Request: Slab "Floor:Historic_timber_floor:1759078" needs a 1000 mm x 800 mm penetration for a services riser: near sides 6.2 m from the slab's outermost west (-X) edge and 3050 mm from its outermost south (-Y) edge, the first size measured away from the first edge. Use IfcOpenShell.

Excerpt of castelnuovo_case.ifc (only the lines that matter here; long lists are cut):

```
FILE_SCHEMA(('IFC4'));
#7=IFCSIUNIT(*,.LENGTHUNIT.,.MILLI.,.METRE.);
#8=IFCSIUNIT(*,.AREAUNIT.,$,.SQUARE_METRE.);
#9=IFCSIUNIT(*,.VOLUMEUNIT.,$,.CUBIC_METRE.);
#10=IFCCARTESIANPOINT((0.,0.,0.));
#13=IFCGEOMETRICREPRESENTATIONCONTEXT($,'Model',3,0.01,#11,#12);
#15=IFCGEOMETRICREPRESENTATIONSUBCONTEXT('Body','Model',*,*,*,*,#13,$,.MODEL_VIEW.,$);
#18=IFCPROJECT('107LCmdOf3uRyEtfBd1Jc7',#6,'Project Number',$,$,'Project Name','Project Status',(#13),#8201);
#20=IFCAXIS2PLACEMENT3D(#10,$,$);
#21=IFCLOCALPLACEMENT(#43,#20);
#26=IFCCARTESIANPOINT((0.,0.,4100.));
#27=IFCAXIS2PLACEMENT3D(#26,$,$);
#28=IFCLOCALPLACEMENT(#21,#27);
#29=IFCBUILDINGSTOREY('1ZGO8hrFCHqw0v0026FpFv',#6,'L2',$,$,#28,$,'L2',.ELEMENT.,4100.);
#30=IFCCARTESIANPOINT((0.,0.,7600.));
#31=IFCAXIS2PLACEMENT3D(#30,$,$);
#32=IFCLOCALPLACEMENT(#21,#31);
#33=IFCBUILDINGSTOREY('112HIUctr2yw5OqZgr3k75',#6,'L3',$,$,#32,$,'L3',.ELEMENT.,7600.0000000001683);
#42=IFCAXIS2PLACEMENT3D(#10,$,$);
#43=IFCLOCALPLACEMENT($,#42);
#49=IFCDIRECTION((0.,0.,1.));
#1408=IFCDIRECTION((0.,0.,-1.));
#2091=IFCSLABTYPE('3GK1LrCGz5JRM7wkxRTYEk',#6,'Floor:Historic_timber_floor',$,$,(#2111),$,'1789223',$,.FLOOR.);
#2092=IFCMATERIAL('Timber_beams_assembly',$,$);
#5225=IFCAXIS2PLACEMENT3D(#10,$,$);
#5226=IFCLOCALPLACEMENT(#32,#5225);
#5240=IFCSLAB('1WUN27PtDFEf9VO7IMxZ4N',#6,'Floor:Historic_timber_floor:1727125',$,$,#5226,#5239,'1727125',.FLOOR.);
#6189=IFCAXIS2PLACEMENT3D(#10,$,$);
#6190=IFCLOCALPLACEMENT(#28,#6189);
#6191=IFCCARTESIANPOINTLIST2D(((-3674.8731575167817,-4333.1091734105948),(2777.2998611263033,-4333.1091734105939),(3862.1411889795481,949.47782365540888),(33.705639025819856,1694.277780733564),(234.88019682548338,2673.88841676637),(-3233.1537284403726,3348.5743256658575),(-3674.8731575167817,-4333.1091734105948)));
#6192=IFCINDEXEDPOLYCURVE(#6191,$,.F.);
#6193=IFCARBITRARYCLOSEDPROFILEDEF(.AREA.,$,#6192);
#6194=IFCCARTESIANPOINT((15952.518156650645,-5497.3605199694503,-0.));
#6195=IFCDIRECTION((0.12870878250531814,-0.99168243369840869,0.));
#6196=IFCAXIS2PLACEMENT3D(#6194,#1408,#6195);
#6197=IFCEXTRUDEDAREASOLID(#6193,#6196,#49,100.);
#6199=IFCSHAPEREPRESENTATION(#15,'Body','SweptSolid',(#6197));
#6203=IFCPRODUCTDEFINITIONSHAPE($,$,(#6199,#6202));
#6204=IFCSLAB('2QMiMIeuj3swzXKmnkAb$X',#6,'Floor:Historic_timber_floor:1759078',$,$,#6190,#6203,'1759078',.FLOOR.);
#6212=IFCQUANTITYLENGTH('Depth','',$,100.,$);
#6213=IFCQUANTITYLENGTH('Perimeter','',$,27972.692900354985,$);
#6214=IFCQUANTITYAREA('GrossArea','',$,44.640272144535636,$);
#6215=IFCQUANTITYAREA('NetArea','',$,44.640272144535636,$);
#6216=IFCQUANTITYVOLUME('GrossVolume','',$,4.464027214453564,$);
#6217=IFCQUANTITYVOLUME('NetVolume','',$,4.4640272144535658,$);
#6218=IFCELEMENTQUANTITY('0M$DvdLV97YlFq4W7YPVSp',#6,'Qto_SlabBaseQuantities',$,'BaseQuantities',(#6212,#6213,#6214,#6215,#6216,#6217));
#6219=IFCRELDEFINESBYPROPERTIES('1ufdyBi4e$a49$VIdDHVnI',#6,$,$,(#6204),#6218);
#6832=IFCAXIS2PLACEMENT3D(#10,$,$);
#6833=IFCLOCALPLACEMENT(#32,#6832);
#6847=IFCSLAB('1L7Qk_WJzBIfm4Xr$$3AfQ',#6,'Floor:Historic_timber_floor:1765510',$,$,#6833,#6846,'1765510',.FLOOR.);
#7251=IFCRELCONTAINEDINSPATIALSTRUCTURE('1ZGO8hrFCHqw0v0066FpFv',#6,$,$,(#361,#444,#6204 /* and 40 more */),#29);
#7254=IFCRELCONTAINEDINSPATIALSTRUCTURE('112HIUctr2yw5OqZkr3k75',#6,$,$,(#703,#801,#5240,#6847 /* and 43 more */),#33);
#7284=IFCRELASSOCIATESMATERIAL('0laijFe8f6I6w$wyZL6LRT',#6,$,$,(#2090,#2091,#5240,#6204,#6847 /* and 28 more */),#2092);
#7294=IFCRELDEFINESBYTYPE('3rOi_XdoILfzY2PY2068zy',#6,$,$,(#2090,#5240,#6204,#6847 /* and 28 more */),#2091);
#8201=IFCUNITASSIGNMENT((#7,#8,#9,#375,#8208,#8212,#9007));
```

```python
import numpy as np
import ifcopenshell
import ifcopenshell.api.feature
import ifcopenshell.api.geometry
import ifcopenshell.api.pset
import ifcopenshell.api.root
import ifcopenshell.geom
import ifcopenshell.util.element
import ifcopenshell.util.placement
import ifcopenshell.util.representation
import ifcopenshell.util.shape
import ifcopenshell.util.unit

model = ifcopenshell.open("castelnuovo_case.ifc")
unit_scale = ifcopenshell.util.unit.calculate_unit_scale(model)
area_scale = ifcopenshell.util.unit.calculate_unit_scale(model, "AREAUNIT")
volume_scale = ifcopenshell.util.unit.calculate_unit_scale(model, "VOLUMEUNIT")
settings = ifcopenshell.geom.settings()


def volume(element):
    """Net volume in cubic metres, openings subtracted."""
    shape = ifcopenshell.geom.create_shape(settings, element)
    return ifcopenshell.util.shape.get_volume(shape.geometry)


slab = model.by_guid("2QMiMIeuj3swzXKmnkAb$X")
before = volume(slab)

# Extent in the slab's own axes, in metres. The edges named are its -X and -Y sides.
slab_shape = ifcopenshell.geom.create_shape(settings, slab)
vertices = ifcopenshell.util.shape.get_vertices(slab_shape.geometry)
x_min, y_min, bottom = vertices.min(axis=0)
top = vertices[:, 2].max()

opening = ifcopenshell.api.root.create_entity(model, ifc_class="IfcOpeningElement", name="Services riser opening", predefined_type="OPENING")
context = ifcopenshell.util.representation.get_context(model, "Model", "Body", "MODEL_VIEW")
width, depth = 1, 0.8
outline = [(0.0, 0.0), (width, 0.0), (width, depth), (0.0, depth), (0.0, 0.0)]
# Overshoot both faces by 50 mm so the cut is clean.
shape = ifcopenshell.api.geometry.add_slab_representation(
    model, context=context, depth=top - bottom + 0.1, polyline=outline
)
ifcopenshell.api.geometry.assign_representation(model, product=opening, representation=shape)

matrix = ifcopenshell.util.placement.get_local_placement(slab.ObjectPlacement)
matrix[:, 3] = matrix @ np.append(np.array([x_min + 6.2, y_min + 3.05, bottom - 0.05]) / unit_scale, 1.0)
ifcopenshell.api.geometry.edit_object_placement(model, product=opening, matrix=matrix, is_si=False)
ifcopenshell.api.feature.add_feature(model, feature=opening, element=slab)

after = volume(slab)

# Update the slab's stored quantities.
qto = model.by_id(ifcopenshell.util.element.get_pset(slab, "Qto_SlabBaseQuantities", should_inherit=False)["id"])
ifcopenshell.api.pset.edit_qto(model, qto=qto, properties={
    "NetArea": after / (top - bottom) / area_scale,
    "NetVolume": after / volume_scale,
})

print(f"slab volume {before:.3f} -> {after:.3f} m3")

model.write("castelnuovo_case_updated.ifc")
```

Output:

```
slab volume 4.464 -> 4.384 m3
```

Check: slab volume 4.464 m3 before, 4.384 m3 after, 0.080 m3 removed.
